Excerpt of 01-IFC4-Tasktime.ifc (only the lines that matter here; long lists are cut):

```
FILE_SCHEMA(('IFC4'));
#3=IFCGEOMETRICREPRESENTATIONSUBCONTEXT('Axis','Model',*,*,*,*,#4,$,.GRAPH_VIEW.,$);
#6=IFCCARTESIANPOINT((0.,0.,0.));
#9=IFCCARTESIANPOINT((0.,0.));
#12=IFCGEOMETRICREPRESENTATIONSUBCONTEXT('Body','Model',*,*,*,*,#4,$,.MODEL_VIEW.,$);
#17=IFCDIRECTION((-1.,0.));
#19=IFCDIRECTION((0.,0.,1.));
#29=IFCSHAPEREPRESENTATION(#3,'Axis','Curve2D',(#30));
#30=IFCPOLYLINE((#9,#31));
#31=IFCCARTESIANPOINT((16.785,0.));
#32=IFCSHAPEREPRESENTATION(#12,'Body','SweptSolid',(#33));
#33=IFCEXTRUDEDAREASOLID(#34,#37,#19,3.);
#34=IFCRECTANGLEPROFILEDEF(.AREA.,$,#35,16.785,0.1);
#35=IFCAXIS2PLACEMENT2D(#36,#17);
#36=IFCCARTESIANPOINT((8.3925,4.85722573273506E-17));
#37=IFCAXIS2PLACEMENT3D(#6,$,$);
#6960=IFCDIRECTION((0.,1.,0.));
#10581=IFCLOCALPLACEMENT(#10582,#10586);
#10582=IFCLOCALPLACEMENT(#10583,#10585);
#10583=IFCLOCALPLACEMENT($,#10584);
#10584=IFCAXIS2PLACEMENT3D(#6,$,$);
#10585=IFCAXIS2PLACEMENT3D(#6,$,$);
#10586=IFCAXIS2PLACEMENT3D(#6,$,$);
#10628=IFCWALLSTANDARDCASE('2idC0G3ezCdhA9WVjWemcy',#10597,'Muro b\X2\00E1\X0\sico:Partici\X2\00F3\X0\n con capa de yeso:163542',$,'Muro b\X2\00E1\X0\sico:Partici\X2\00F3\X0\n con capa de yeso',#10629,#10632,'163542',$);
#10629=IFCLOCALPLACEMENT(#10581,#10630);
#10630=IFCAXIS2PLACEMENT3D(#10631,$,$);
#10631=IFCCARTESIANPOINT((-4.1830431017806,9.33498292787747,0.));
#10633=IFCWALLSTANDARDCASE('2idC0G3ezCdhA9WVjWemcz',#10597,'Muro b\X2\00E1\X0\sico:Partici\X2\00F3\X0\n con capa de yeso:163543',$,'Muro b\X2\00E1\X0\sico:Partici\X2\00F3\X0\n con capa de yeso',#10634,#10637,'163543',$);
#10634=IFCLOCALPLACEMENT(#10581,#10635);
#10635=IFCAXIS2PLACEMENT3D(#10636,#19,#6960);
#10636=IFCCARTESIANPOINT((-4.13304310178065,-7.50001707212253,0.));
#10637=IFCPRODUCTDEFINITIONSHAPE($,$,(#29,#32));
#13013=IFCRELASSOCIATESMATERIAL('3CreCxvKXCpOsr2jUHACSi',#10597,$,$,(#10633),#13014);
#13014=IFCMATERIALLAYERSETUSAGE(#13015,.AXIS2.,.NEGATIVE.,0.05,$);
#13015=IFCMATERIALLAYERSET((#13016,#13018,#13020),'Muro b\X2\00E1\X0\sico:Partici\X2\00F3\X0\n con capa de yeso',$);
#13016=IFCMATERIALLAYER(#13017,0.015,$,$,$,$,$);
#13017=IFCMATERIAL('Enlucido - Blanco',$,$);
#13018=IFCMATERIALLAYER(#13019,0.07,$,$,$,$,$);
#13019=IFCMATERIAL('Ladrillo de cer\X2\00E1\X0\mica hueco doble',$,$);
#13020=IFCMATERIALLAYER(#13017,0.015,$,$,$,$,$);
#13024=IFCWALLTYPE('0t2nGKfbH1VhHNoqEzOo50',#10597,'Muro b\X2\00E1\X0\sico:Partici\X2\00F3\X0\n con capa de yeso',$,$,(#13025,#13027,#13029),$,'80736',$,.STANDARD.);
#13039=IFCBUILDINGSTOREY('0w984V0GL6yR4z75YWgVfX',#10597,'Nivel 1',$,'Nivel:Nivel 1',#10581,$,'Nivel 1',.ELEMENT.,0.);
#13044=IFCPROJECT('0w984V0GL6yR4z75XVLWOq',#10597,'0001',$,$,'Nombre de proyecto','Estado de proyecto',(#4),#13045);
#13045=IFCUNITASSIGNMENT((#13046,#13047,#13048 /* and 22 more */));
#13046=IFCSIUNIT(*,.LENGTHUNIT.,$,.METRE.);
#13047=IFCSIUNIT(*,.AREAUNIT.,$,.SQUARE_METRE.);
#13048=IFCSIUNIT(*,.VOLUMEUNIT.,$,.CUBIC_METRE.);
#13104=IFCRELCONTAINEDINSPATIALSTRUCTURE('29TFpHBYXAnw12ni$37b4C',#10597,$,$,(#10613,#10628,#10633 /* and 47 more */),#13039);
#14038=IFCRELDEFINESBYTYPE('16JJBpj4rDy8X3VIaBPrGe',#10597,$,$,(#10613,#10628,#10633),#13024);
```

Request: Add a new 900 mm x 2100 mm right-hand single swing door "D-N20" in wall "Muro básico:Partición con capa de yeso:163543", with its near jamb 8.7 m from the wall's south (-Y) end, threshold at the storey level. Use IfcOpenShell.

```python
import numpy as np
import ifcopenshell
import ifcopenshell.api.feature
import ifcopenshell.api.geometry
import ifcopenshell.api.root
import ifcopenshell.api.spatial
import ifcopenshell.geom
import ifcopenshell.util.element
import ifcopenshell.util.placement
import ifcopenshell.util.representation
import ifcopenshell.util.shape
import ifcopenshell.util.unit

model = ifcopenshell.open("01-IFC4-Tasktime.ifc")
unit_scale = ifcopenshell.util.unit.calculate_unit_scale(model)
settings = ifcopenshell.geom.settings()


def volume(element):
    """Net volume in cubic metres, openings subtracted."""
    shape = ifcopenshell.geom.create_shape(settings, element)
    return ifcopenshell.util.shape.get_volume(shape.geometry)


wall = model.by_id(10633)
storey = ifcopenshell.util.element.get_container(wall, ifc_class="IfcBuildingStorey")
context = ifcopenshell.util.representation.get_context(model, "Model", "Body", "MODEL_VIEW")
before = volume(wall)

width, height, from_end, sill = 0.9, 2.1, 8.7, 0.0  # metres

# The wall runs along its own X axis, and the end named is its -X end.
wall_shape = ifcopenshell.geom.create_shape(settings, wall)
x, y, z = ifcopenshell.util.shape.get_vertices(wall_shape.geometry).T
start = x.min() + from_end
face, thickness = float(y.min()), float(y.max() - y.min())
wall_matrix = ifcopenshell.util.placement.get_local_placement(wall.ObjectPlacement)
level = ifcopenshell.util.placement.get_local_placement(storey.ObjectPlacement)[2, 3]


def in_wall(x, y):
    """Placement at x, y metres in the wall's axes, at sill height."""
    matrix = wall_matrix.copy()
    matrix[:, 3] = wall_matrix @ np.array([x / unit_scale, y / unit_scale, 0.0, 1.0])
    matrix[2, 3] = level + sill / unit_scale
    return matrix


# Opening: a box that overshoots both wall faces by 50 mm.
opening = ifcopenshell.api.root.create_entity(model, ifc_class="IfcOpeningElement", predefined_type="OPENING")
box = ifcopenshell.api.geometry.add_wall_representation(
    model, context=context, length=width, height=height, thickness=thickness + 0.1
)
ifcopenshell.api.geometry.assign_representation(model, product=opening, representation=box)
ifcopenshell.api.geometry.edit_object_placement(model, product=opening, matrix=in_wall(start, face - 0.05), is_si=False)
ifcopenshell.api.feature.add_feature(model, feature=opening, element=wall)

door = ifcopenshell.api.root.create_entity(model, ifc_class="IfcDoor", name="D-N20", predefined_type="DOOR")
door.OverallWidth, door.OverallHeight = width / unit_scale, height / unit_scale
door.OperationType = "SINGLE_SWING_RIGHT"
body = ifcopenshell.api.geometry.add_door_representation(
    model,
    context=context,
    overall_width=door.OverallWidth,
    overall_height=door.OverallHeight,
    operation_type="SINGLE_SWING_RIGHT",
    lining_properties={"LiningDepth": thickness / unit_scale, "ThresholdDepth": thickness / unit_scale},
)
ifcopenshell.api.geometry.assign_representation(model, product=door, representation=body)
ifcopenshell.api.spatial.assign_container(model, products=[door], relating_structure=storey)
ifcopenshell.api.feature.add_filling(model, opening=opening, element=door)

# The lining spans the wall, so the door starts at the wall face.
ifcopenshell.api.geometry.edit_object_placement(model, product=door, matrix=in_wall(start, face), is_si=False)

after = volume(wall)

print(f"wall volume {before:.3f} -> {after:.3f} m3")

model.write("01-IFC4-Tasktime_edited.ifc")
```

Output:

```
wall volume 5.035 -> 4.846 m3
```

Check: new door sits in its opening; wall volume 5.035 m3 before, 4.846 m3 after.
